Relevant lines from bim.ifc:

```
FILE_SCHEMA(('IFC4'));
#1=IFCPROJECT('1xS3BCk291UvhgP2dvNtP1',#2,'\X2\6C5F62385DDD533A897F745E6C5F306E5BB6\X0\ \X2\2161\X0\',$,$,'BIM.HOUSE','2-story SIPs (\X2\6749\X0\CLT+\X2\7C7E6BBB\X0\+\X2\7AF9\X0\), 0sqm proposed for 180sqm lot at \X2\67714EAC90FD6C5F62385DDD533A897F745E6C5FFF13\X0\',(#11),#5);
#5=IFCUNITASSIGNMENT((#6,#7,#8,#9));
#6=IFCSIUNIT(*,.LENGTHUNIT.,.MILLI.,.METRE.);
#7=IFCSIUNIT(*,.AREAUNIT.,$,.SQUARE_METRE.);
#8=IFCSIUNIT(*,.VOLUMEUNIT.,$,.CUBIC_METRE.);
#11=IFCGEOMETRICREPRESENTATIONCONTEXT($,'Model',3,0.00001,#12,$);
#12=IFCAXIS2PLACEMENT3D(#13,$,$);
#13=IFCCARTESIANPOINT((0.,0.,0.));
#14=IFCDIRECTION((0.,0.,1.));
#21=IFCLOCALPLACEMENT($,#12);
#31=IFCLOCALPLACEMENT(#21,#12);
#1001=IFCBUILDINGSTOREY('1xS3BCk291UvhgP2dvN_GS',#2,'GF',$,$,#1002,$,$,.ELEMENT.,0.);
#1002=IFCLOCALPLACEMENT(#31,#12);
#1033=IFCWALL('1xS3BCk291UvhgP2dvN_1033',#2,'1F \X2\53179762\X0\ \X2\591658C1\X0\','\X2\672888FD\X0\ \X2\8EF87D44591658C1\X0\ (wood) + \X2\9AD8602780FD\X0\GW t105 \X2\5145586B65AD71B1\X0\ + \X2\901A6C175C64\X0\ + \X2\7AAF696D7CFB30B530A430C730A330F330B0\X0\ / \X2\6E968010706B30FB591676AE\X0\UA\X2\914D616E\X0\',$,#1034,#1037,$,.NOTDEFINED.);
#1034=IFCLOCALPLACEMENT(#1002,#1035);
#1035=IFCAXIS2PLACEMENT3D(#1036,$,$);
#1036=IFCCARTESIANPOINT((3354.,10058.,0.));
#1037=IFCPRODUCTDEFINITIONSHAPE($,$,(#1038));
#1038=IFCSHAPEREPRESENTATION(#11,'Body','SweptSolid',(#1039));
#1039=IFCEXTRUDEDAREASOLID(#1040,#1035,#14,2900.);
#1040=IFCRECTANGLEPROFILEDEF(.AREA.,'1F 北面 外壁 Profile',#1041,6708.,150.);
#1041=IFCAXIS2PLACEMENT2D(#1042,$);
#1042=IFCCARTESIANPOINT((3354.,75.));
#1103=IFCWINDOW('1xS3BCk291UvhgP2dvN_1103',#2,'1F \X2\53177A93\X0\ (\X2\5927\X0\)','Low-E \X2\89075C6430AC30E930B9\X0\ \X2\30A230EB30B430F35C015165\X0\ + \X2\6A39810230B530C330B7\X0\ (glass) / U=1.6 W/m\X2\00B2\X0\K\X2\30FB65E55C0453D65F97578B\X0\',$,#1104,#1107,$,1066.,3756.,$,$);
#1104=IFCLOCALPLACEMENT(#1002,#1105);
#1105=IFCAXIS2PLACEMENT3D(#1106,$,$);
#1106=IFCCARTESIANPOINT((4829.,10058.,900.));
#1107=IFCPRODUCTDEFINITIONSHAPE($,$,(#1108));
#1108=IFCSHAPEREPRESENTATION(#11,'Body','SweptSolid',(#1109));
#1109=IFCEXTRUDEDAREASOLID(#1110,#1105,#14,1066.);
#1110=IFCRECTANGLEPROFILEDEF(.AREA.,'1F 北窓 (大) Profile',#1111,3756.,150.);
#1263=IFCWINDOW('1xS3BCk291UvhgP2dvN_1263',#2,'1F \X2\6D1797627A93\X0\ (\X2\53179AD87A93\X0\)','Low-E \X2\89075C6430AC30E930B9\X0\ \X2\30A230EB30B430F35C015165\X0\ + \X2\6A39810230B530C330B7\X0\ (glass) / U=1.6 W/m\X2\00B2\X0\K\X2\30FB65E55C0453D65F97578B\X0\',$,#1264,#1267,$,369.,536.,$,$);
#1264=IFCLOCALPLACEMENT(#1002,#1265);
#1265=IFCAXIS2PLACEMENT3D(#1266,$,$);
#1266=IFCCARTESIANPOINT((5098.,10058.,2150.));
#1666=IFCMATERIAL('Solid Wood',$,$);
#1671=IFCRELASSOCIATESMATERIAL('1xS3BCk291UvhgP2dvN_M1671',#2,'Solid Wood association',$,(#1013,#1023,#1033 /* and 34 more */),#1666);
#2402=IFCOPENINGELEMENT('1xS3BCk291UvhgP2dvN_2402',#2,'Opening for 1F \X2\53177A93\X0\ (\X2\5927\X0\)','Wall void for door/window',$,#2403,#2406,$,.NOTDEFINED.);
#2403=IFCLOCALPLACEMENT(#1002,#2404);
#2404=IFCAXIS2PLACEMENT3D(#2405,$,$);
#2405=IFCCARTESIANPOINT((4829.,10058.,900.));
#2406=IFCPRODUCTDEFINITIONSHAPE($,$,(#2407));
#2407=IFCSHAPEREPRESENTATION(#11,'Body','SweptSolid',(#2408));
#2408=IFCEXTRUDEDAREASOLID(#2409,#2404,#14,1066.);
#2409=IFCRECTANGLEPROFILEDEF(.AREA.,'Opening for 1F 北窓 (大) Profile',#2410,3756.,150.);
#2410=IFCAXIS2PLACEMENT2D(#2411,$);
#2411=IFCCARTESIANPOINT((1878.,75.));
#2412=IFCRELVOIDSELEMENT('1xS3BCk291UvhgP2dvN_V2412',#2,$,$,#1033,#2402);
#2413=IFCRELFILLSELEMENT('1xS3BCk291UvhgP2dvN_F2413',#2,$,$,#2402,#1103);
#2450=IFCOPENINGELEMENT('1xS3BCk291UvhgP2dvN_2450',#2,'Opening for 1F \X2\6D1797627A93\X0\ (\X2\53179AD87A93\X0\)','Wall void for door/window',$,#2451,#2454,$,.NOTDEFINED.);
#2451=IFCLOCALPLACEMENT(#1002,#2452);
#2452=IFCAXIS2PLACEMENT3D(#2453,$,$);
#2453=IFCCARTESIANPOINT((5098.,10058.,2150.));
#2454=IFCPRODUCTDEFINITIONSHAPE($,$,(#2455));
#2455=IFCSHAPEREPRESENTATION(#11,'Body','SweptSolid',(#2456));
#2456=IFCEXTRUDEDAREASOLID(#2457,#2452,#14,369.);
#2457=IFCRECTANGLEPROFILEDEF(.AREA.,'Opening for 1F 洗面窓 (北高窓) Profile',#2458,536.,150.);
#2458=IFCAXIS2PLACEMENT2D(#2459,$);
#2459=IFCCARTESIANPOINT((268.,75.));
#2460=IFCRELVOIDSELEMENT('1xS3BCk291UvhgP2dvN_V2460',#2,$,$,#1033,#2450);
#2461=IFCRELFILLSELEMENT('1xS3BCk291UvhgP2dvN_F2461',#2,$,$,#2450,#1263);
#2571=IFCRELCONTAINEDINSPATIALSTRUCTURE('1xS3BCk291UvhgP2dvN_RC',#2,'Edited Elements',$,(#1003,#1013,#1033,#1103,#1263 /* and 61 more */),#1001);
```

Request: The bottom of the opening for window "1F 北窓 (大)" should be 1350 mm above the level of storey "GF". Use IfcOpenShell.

```python
import numpy as np
import ifcopenshell
import ifcopenshell.api.geometry
import ifcopenshell.geom
import ifcopenshell.util.element
import ifcopenshell.util.placement
import ifcopenshell.util.shape
import ifcopenshell.util.unit

model = ifcopenshell.open("bim.ifc")
unit_scale = ifcopenshell.util.unit.calculate_unit_scale(model)

window = model.by_id(1103)
opening = window.FillsVoids[0].RelatingOpeningElement
storey = ifcopenshell.util.element.get_container(window, ifc_class="IfcBuildingStorey")
level = ifcopenshell.util.placement.get_local_placement(storey.ObjectPlacement)[2, 3]

# The opening's origin need not be at the sill, so measure its lowest point.
shape = ifcopenshell.geom.create_shape(ifcopenshell.geom.settings(), opening)
bottom = ifcopenshell.util.shape.get_shape_bottom_elevation(shape, shape.geometry) / unit_scale
dz = level + 1350.0 - bottom

shift = np.array([0.0, 0.0, dz])
# The window is not placed relative to its opening, so move both.
for product in (opening, window):
    matrix = ifcopenshell.util.placement.get_local_placement(product.ObjectPlacement)
    matrix[:3, 3] += shift
    ifcopenshell.api.geometry.edit_object_placement(model, product=product, matrix=matrix, is_si=False)

print(f"moved by {dz * unit_scale:+.3f} m")

model.write("bim_updated.ifc")
```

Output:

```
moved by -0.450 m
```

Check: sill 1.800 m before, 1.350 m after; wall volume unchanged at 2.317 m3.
